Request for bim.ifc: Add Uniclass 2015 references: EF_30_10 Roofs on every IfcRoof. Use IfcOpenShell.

First a look at what the model holds.

```python
import ifcopenshell

model = ifcopenshell.open("bim.ifc")
print(model.schema)
print("classifications:", [c.Name for c in model.by_type("IfcClassification")])
for ifc_class in ("IfcDoor", "IfcRoof", "IfcStair", "IfcWall", "IfcWindow"):
    print(ifc_class, len(model.by_type(ifc_class)))
```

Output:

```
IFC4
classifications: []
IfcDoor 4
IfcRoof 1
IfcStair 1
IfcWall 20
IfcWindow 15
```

```python
import ifcopenshell
import ifcopenshell.api.classification

model = ifcopenshell.open("bim.ifc")

system = ifcopenshell.api.classification.add_classification(model, classification="Uniclass 2015")

codes = {
    "IfcRoof": ("EF_30_10", "Roofs"),
}
for ifc_class, (code, name) in codes.items():
    products = model.by_type(ifc_class)
    ifcopenshell.api.classification.add_reference(
        model, products=products, classification=system, identification=code, name=name
    )
    print(code, len(products))

model.write("bim_updated.ifc")
```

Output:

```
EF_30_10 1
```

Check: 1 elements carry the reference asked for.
